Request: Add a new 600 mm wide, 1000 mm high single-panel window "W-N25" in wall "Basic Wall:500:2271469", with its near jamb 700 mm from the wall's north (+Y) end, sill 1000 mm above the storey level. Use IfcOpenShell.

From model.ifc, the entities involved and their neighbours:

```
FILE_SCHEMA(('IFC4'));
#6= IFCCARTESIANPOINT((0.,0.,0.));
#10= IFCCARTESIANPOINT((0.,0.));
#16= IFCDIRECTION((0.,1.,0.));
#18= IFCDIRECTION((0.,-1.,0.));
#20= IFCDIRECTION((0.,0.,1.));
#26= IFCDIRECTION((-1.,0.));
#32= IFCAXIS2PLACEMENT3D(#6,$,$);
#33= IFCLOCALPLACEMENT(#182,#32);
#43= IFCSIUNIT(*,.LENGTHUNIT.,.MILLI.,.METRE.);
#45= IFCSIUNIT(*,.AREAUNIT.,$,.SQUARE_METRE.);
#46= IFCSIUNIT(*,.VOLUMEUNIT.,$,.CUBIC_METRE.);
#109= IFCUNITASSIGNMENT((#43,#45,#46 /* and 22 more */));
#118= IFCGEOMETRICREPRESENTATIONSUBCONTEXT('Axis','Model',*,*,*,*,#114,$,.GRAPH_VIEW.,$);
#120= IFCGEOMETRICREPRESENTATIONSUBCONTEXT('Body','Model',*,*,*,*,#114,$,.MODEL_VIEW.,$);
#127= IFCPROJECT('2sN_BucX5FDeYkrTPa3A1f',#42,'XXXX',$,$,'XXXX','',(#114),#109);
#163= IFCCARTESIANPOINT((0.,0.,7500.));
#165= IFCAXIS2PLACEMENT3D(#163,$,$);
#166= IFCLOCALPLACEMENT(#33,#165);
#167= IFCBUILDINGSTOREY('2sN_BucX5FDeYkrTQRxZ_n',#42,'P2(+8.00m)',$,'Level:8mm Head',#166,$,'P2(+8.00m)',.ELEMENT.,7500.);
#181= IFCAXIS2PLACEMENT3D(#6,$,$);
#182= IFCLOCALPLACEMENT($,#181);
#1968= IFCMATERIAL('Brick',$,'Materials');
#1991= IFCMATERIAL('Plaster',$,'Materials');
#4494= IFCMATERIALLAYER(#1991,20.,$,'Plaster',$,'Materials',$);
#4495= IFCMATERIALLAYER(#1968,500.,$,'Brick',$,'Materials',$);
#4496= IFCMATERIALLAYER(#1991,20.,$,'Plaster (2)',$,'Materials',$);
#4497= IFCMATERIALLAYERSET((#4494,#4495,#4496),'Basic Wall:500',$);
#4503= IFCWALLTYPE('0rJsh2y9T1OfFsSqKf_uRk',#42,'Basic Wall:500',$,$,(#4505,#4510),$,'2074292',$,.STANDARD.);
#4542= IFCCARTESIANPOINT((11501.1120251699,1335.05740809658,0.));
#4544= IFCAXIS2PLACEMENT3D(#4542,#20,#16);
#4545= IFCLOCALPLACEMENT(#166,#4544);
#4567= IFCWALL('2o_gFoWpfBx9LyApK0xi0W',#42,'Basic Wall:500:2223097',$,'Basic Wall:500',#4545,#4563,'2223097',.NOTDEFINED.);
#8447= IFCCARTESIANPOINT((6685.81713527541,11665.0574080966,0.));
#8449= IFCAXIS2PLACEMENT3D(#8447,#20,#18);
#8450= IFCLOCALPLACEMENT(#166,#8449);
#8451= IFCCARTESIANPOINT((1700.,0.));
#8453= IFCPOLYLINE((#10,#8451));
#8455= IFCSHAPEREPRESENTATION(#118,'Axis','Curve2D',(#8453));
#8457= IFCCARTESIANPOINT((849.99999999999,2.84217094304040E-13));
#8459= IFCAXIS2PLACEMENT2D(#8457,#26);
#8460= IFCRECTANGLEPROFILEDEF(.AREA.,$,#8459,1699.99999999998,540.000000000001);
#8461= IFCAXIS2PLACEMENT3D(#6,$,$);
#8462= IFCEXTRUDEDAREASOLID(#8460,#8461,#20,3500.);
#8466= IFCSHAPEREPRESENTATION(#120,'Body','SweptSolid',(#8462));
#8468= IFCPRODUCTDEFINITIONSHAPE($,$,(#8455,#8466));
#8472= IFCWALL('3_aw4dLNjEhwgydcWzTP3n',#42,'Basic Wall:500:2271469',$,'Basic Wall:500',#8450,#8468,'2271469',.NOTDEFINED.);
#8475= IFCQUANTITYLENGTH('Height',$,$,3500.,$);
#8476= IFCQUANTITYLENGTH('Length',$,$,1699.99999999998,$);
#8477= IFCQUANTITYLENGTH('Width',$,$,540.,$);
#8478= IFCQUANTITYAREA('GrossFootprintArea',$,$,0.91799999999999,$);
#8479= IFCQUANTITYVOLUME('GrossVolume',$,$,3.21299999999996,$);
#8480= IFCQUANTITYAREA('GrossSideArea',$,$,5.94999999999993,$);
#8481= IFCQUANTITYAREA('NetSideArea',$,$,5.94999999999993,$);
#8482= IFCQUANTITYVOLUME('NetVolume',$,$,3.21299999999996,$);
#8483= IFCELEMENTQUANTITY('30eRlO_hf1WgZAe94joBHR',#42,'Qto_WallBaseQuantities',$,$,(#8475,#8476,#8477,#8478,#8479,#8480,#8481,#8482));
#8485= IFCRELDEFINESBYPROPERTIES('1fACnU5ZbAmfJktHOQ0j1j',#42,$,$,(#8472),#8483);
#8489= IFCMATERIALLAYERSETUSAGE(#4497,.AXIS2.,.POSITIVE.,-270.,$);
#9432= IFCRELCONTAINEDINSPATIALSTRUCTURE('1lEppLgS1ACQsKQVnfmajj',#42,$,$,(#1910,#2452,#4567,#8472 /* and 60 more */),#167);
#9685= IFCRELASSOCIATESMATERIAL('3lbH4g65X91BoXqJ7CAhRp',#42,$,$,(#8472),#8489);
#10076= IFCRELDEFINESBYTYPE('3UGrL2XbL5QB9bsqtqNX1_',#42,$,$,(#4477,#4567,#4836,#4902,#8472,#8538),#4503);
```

```python
import numpy as np
import ifcopenshell
import ifcopenshell.api.feature
import ifcopenshell.api.geometry
import ifcopenshell.api.pset
import ifcopenshell.api.root
import ifcopenshell.api.spatial
import ifcopenshell.geom
import ifcopenshell.util.element
import ifcopenshell.util.placement
import ifcopenshell.util.representation
import ifcopenshell.util.shape
import ifcopenshell.util.unit

model = ifcopenshell.open("model.ifc")
unit_scale = ifcopenshell.util.unit.calculate_unit_scale(model)
area_scale = ifcopenshell.util.unit.calculate_unit_scale(model, "AREAUNIT")
volume_scale = ifcopenshell.util.unit.calculate_unit_scale(model, "VOLUMEUNIT")
settings = ifcopenshell.geom.settings()


def volume(element):
    """Net volume in cubic metres, openings subtracted."""
    shape = ifcopenshell.geom.create_shape(settings, element)
    return ifcopenshell.util.shape.get_volume(shape.geometry)


wall = model.by_id(8472)
storey = ifcopenshell.util.element.get_container(wall, ifc_class="IfcBuildingStorey")
context = ifcopenshell.util.representation.get_context(model, "Model", "Body", "MODEL_VIEW")
before = volume(wall)

width, height, from_end, sill = 0.6, 1, 0.7, 1  # metres

# The wall runs along its own X axis, and the end named is its -X end.
wall_shape = ifcopenshell.geom.create_shape(settings, wall)
x, y, z = ifcopenshell.util.shape.get_vertices(wall_shape.geometry).T
start = x.min() + from_end
face, thickness = float(y.min()), float(y.max() - y.min())
wall_matrix = ifcopenshell.util.placement.get_local_placement(wall.ObjectPlacement)
level = ifcopenshell.util.placement.get_local_placement(storey.ObjectPlacement)[2, 3]


def in_wall(x, y):
    """Placement at x, y metres in the wall's axes, at sill height."""
    matrix = wall_matrix.copy()
    matrix[:, 3] = wall_matrix @ np.array([x / unit_scale, y / unit_scale, 0.0, 1.0])
    matrix[2, 3] = level + sill / unit_scale
    return matrix


# Opening: a box that overshoots both wall faces by 50 mm.
opening = ifcopenshell.api.root.create_entity(model, ifc_class="IfcOpeningElement", predefined_type="OPENING")
box = ifcopenshell.api.geometry.add_wall_representation(
    model, context=context, length=width, height=height, thickness=thickness + 0.1
)
ifcopenshell.api.geometry.assign_representation(model, product=opening, representation=box)
ifcopenshell.api.geometry.edit_object_placement(model, product=opening, matrix=in_wall(start, face - 0.05), is_si=False)
ifcopenshell.api.feature.add_feature(model, feature=opening, element=wall)

window = ifcopenshell.api.root.create_entity(model, ifc_class="IfcWindow", name="W-N25", predefined_type="WINDOW")
window.OverallWidth, window.OverallHeight = width / unit_scale, height / unit_scale
window.PartitioningType = "SINGLE_PANEL"
body = ifcopenshell.api.geometry.add_window_representation(
    model,
    context=context,
    overall_width=window.OverallWidth,
    overall_height=window.OverallHeight,
    partition_type="SINGLE_PANEL",
)
ifcopenshell.api.geometry.assign_representation(model, product=window, representation=body)
ifcopenshell.api.spatial.assign_container(model, products=[window], relating_structure=storey)
ifcopenshell.api.feature.add_filling(model, opening=opening, element=window)

# Centre the window in the wall's thickness.
ifcopenshell.api.geometry.edit_object_placement(model, product=window, matrix=in_wall(start, face), is_si=False)
window_shape = ifcopenshell.geom.create_shape(settings, window)
depth = ifcopenshell.util.shape.get_vertices(window_shape.geometry)[:, 1]
offset = face + thickness / 2 - (depth.min() + depth.max()) / 2
ifcopenshell.api.geometry.edit_object_placement(model, product=window, matrix=in_wall(start, offset), is_si=False)

after = volume(wall)

# Update the wall's stored quantities.
qto = model.by_id(ifcopenshell.util.element.get_pset(wall, "Qto_WallBaseQuantities", should_inherit=False)["id"])
ifcopenshell.api.pset.edit_qto(model, qto=qto, properties={
    "NetSideArea": after / thickness / area_scale,
    "NetVolume": after / volume_scale,
})

print(f"wall volume {before:.3f} -> {after:.3f} m3")

model.write("model_updated.ifc")
```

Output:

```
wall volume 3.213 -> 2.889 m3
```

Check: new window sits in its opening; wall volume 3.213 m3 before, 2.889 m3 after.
